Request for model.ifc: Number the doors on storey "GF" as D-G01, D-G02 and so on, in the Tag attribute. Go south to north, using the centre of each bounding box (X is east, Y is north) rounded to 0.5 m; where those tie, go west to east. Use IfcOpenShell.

First a look at what the model holds.

```python
import ifcopenshell
import ifcopenshell.util.element
import ifcopenshell.util.placement

model = ifcopenshell.open("model.ifc")
print(model.schema)
storey = next(s for s in model.by_type("IfcBuildingStorey") if s.Name == "GF")
doors = [e for e in ifcopenshell.util.element.get_decomposition(storey) if e.is_a("IfcDoor")]
for e in sorted(doors, key=lambda e: e.id()):
    origin = ifcopenshell.util.placement.get_local_placement(e.ObjectPlacement)[:3, 3]
    print(e.id(), e.Tag, e.Name, origin.round(2) + 0.0, sep=" | ")
```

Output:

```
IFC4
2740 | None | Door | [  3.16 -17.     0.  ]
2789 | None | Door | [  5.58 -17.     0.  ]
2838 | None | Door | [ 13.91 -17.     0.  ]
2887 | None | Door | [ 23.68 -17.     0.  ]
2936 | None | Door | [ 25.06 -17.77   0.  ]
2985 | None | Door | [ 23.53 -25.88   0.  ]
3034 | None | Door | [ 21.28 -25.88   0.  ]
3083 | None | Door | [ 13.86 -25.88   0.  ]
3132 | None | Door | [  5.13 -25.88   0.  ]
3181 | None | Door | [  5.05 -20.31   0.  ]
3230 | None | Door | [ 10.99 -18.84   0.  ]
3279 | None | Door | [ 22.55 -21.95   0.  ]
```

```python
import ifcopenshell
import ifcopenshell.geom
import ifcopenshell.util.element
import ifcopenshell.util.shape

model = ifcopenshell.open("model.ifc")
settings = ifcopenshell.geom.settings()
settings.set("use-world-coords", True)


def centre(element):
    shape = ifcopenshell.geom.create_shape(settings, element)
    return ifcopenshell.util.shape.get_bbox_centroid(shape.geometry)


storey = next(s for s in model.by_type("IfcBuildingStorey") if s.Name == "GF")
doors = [e for e in ifcopenshell.util.element.get_decomposition(storey) if e.is_a("IfcDoor")]

# Insertion points can sit at a corner or the storey origin, so sort by the geometry (in metres).
centres = {e: centre(e) for e in doors}
doors.sort(key=lambda e: (round(centres[e][1] / 0.5), centres[e][0]))

for i, e in enumerate(doors, start=1):
    number = f"D-G{i:02d}"
    e.Tag = number
    print(e.id(), number)

model.write("model-out.ifc")
```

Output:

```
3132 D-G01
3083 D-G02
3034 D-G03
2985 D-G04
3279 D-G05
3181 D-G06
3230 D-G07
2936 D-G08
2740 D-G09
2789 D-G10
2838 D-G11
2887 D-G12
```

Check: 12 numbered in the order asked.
